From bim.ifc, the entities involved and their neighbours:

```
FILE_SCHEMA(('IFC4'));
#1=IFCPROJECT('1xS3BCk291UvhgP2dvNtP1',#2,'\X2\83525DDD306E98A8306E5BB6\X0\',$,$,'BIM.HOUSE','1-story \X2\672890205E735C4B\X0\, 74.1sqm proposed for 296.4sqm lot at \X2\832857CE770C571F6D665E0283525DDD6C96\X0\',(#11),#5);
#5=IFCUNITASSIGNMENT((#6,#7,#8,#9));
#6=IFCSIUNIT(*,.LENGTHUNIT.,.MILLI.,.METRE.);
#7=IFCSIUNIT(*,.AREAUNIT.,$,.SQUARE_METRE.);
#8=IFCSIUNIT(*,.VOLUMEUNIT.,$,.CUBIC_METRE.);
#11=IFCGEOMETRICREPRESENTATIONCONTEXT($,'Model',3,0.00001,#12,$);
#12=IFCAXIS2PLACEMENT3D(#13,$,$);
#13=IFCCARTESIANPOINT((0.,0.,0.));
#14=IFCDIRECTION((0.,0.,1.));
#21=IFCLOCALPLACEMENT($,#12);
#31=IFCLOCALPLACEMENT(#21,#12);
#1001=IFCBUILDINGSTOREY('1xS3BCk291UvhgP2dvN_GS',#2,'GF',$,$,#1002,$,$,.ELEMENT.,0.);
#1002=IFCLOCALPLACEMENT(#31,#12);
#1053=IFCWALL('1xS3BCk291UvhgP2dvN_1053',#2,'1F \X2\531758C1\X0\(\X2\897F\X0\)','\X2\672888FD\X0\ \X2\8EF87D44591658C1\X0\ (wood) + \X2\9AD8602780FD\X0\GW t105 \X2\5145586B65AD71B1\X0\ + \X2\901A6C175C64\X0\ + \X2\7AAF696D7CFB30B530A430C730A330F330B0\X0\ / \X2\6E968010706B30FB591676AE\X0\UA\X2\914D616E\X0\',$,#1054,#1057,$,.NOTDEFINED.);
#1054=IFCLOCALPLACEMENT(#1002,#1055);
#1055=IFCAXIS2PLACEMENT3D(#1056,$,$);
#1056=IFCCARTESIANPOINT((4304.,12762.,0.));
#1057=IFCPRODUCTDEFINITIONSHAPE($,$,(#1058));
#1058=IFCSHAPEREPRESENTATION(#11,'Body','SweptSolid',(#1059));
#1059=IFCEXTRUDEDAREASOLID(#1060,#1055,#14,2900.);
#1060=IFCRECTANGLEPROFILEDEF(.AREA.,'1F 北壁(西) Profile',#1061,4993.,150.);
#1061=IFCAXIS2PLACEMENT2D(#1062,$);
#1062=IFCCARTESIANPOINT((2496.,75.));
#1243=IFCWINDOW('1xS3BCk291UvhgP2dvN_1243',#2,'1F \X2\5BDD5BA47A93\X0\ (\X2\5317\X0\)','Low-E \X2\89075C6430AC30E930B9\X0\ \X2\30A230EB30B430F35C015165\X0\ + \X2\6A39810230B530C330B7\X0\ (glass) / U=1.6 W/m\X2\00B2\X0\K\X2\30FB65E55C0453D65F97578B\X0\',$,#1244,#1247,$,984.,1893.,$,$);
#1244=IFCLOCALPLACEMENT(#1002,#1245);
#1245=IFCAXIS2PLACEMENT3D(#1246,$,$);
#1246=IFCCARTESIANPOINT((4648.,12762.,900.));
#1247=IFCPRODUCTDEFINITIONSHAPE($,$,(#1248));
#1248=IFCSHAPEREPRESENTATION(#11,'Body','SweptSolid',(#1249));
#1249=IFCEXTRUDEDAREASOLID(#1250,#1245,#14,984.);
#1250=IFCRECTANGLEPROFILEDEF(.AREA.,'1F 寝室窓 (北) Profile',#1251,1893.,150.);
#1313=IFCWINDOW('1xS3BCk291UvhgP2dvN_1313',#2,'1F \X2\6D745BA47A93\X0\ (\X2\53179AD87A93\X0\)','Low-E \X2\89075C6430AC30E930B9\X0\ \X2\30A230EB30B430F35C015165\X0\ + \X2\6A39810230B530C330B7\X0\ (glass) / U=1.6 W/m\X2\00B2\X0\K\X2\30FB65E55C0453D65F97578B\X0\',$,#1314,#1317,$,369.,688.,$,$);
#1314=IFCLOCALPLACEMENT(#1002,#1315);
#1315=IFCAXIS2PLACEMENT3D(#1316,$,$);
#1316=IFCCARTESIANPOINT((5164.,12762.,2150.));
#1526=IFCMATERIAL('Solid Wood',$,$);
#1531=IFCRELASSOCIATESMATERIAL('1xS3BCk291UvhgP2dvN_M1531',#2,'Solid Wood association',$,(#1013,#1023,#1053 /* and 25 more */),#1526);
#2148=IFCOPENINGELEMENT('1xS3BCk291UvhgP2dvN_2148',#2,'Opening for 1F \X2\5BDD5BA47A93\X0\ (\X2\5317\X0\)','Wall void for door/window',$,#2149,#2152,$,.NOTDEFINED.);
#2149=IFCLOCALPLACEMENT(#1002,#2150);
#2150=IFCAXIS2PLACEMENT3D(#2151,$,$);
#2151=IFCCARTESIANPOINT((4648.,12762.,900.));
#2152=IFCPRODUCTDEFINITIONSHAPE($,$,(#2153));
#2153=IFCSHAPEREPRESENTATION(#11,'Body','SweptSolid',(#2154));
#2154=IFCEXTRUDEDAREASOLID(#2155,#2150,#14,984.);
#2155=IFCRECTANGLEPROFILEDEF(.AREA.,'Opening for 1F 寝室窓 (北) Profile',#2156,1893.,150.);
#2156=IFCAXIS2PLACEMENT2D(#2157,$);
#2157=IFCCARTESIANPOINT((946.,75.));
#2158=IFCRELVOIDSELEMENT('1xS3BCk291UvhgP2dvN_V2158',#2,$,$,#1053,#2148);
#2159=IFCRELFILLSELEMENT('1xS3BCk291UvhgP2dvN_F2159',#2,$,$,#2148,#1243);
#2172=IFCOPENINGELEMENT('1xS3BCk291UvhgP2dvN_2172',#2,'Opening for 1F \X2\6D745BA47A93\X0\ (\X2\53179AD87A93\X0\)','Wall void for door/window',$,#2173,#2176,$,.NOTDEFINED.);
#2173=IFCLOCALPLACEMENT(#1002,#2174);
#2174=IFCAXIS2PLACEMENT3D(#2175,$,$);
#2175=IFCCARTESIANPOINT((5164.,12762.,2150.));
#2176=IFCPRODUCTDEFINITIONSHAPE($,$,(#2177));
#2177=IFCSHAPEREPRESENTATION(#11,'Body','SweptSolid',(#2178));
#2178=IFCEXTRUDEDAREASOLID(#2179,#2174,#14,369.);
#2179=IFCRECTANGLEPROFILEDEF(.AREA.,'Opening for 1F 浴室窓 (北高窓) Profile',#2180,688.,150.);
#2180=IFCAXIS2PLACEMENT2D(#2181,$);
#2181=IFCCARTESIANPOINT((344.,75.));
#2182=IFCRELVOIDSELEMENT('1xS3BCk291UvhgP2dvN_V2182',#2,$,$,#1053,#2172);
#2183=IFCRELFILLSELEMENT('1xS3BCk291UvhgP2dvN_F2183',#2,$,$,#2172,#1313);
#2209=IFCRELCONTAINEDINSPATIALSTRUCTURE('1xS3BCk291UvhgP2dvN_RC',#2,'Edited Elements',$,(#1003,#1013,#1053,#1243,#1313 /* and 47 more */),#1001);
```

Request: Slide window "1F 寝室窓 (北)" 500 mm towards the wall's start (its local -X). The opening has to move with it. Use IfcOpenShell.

```python
import ifcopenshell
import ifcopenshell.api.geometry
import ifcopenshell.util.placement
import ifcopenshell.util.unit

model = ifcopenshell.open("bim.ifc")
unit_scale = ifcopenshell.util.unit.calculate_unit_scale(model)

window = model.by_guid("1xS3BCk291UvhgP2dvN_1243")
opening = window.FillsVoids[0].RelatingOpeningElement
wall = opening.VoidsElements[0].RelatingBuildingElement

wall_matrix = ifcopenshell.util.placement.get_local_placement(wall.ObjectPlacement)
shift = wall_matrix[:3, 0] * -0.5 / unit_scale
before = ifcopenshell.util.placement.get_local_placement(window.ObjectPlacement)[:3, 3].copy()

# The window is not placed relative to its opening, so move both.
for product in (opening, window):
    matrix = ifcopenshell.util.placement.get_local_placement(product.ObjectPlacement)
    matrix[:3, 3] += shift
    ifcopenshell.api.geometry.edit_object_placement(model, product=product, matrix=matrix, is_si=False)

after = ifcopenshell.util.placement.get_local_placement(window.ObjectPlacement)[:3, 3]
print("window moved by", (after - before).round(3) + 0.0)

model.write("bim-out.ifc")
```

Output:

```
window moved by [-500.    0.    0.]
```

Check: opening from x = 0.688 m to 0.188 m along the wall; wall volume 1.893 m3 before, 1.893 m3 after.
